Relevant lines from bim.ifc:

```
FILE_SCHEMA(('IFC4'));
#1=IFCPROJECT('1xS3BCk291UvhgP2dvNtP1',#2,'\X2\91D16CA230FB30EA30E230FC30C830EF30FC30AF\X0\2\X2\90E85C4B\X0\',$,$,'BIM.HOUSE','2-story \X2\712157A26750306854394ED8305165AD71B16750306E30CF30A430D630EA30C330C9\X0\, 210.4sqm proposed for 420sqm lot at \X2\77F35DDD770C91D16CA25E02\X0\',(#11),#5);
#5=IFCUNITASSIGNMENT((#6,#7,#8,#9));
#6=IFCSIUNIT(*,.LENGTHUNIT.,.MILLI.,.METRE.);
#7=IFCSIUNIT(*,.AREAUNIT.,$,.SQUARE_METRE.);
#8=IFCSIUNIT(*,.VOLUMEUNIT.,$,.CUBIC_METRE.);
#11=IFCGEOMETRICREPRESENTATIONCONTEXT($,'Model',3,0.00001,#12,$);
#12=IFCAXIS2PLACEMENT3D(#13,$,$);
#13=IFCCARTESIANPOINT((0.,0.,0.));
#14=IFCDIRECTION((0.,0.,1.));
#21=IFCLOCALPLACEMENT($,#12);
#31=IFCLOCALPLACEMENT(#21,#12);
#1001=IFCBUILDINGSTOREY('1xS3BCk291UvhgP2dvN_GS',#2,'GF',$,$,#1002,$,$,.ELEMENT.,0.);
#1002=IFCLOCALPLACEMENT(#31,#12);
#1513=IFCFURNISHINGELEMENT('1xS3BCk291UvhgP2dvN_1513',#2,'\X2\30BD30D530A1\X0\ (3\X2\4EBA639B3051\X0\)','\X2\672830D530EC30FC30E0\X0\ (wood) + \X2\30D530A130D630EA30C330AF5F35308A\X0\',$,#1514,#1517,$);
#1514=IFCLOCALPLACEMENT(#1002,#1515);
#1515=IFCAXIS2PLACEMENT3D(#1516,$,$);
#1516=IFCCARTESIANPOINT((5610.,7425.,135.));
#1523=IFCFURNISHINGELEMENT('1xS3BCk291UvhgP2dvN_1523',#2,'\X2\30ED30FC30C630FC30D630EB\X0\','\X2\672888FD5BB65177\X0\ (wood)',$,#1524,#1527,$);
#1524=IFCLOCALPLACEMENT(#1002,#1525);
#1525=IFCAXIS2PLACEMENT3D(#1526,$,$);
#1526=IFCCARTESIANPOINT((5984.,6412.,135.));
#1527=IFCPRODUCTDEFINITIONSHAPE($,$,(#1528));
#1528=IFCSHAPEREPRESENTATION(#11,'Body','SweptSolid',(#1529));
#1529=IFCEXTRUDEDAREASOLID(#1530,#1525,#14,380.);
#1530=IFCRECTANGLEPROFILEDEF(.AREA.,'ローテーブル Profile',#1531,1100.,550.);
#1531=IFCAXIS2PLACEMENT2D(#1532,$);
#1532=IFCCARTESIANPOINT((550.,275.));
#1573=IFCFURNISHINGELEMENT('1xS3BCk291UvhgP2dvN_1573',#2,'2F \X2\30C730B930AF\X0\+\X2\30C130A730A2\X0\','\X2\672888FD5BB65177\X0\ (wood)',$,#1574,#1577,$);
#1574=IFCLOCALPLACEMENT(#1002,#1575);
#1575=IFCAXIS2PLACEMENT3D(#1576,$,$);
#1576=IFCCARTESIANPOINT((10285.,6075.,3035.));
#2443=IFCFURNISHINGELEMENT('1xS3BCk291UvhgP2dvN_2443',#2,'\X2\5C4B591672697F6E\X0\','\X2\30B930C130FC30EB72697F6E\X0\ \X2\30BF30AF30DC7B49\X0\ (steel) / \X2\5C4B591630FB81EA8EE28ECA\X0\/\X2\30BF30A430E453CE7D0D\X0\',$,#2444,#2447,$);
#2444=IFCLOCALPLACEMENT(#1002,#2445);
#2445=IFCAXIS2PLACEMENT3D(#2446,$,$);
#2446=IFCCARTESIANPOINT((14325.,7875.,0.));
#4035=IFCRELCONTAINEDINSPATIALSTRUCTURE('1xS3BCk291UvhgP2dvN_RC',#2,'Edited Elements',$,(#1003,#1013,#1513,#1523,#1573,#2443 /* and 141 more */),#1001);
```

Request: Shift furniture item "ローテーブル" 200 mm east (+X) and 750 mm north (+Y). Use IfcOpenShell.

```python
import ifcopenshell
import ifcopenshell.api.geometry
import ifcopenshell.util.placement
import ifcopenshell.util.unit

model = ifcopenshell.open("bim.ifc")
unit_scale = ifcopenshell.util.unit.calculate_unit_scale(model)

item = model.by_id(1523)
matrix = ifcopenshell.util.placement.get_local_placement(item.ObjectPlacement)
matrix[0, 3] += 0.2 / unit_scale
matrix[1, 3] += 0.75 / unit_scale
ifcopenshell.api.geometry.edit_object_placement(model, product=item, matrix=matrix, is_si=False)

print(ifcopenshell.util.placement.get_local_placement(item.ObjectPlacement).round(3) + 0.0)

model.write("bim_updated.ifc")
```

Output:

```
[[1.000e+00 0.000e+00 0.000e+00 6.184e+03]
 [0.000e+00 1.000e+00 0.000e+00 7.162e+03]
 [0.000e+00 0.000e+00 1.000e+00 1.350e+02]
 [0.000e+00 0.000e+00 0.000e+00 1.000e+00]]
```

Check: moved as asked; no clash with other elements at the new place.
